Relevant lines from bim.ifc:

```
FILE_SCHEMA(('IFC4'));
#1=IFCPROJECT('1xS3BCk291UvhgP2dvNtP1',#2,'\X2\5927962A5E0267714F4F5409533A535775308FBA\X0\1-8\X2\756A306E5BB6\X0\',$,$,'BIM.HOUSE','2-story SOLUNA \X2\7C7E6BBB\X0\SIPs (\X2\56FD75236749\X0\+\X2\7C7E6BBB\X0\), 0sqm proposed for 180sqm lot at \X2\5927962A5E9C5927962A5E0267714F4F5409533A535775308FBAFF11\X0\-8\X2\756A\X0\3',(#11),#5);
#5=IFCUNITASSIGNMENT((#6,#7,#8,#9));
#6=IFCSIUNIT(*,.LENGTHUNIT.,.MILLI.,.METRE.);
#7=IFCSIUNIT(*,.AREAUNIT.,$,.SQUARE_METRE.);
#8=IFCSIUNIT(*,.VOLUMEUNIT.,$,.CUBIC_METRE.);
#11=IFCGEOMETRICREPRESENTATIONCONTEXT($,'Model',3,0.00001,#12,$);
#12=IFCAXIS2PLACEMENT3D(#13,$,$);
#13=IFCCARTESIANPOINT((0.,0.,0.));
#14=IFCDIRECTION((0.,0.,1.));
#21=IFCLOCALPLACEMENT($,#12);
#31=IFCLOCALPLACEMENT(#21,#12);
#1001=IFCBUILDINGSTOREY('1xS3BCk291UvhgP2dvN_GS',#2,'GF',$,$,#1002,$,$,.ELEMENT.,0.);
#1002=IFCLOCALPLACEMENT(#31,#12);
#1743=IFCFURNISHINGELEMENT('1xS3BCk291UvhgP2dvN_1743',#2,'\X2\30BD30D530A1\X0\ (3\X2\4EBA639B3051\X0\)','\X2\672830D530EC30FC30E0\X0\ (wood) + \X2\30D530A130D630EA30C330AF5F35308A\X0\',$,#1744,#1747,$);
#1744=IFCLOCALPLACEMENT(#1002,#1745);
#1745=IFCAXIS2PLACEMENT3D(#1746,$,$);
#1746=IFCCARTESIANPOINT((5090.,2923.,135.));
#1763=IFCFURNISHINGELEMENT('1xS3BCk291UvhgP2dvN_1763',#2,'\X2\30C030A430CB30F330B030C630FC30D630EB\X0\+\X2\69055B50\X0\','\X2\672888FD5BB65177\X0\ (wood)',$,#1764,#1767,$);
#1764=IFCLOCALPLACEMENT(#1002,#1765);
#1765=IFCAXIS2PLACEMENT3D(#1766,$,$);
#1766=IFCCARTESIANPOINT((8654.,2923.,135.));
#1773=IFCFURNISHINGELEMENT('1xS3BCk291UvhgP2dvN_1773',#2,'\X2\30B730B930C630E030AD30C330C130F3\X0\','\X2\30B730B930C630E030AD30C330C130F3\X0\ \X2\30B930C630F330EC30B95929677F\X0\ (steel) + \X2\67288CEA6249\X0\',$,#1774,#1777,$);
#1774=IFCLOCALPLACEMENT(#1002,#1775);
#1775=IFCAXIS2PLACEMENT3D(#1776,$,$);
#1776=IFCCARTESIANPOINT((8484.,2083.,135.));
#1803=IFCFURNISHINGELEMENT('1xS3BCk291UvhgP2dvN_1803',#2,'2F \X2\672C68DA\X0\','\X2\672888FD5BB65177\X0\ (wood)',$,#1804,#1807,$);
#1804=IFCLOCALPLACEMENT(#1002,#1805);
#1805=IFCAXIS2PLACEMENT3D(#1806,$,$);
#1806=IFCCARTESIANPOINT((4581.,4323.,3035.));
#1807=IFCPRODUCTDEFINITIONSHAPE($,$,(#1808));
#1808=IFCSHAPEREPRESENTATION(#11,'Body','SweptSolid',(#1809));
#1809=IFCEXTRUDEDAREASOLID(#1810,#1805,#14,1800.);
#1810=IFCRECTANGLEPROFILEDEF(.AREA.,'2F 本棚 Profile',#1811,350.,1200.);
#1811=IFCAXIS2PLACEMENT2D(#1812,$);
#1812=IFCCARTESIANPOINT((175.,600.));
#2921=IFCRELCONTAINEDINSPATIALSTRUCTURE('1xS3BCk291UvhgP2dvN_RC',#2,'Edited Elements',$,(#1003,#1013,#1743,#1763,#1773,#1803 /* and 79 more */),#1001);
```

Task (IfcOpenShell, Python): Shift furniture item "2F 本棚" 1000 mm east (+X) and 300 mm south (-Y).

```python
import ifcopenshell
import ifcopenshell.api.geometry
import ifcopenshell.util.placement

model = ifcopenshell.open("bim.ifc")

item = model.by_id(1803)
matrix = ifcopenshell.util.placement.get_local_placement(item.ObjectPlacement)
matrix[0, 3] += 1000.0
matrix[1, 3] -= 300.0
ifcopenshell.api.geometry.edit_object_placement(model, product=item, matrix=matrix, is_si=False)

print(ifcopenshell.util.placement.get_local_placement(item.ObjectPlacement).round(3) + 0.0)

model.write("bim_v2.ifc")
```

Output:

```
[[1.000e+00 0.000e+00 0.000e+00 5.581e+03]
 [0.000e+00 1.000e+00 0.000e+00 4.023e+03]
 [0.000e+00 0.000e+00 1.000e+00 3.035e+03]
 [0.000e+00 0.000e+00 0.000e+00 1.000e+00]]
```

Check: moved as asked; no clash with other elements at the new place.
